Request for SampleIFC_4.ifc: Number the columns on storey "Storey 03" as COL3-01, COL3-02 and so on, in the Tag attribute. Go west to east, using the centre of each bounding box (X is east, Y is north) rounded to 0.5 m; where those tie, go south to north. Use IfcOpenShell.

First a look at what the model holds.

```python
import ifcopenshell
import ifcopenshell.util.element
import ifcopenshell.util.placement

model = ifcopenshell.open("SampleIFC_4.ifc")
print(model.schema)
storey = next(s for s in model.by_type("IfcBuildingStorey") if s.Name == "Storey 03")
columns = [e for e in ifcopenshell.util.element.get_decomposition(storey) if e.is_a("IfcColumn")]
for e in sorted(columns, key=lambda e: e.id()):
    origin = ifcopenshell.util.placement.get_local_placement(e.ObjectPlacement)[:3, 3]
    print(e.id(), e.Tag, e.Name, origin.round(2) + 0.0, sep=" | ")
```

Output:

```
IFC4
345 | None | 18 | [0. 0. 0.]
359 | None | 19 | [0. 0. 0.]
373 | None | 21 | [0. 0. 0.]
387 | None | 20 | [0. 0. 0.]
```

```python
import ifcopenshell
import ifcopenshell.geom
import ifcopenshell.util.element
import ifcopenshell.util.shape

model = ifcopenshell.open("SampleIFC_4.ifc")
settings = ifcopenshell.geom.settings()
settings.set("use-world-coords", True)


def centre(element):
    shape = ifcopenshell.geom.create_shape(settings, element)
    return ifcopenshell.util.shape.get_bbox_centroid(shape.geometry)


storey = next(s for s in model.by_type("IfcBuildingStorey") if s.Name == "Storey 03")
columns = [e for e in ifcopenshell.util.element.get_decomposition(storey) if e.is_a("IfcColumn")]

# Insertion points can sit at a corner or the storey origin, so sort by the geometry (in metres).
centres = {e: centre(e) for e in columns}
columns.sort(key=lambda e: (round(centres[e][0] / 0.5), centres[e][1]))

for i, e in enumerate(columns, start=1):
    number = f"COL3-{i:02d}"
    e.Tag = number
    print(e.id(), number)

model.write("SampleIFC_4_v2.ifc")
```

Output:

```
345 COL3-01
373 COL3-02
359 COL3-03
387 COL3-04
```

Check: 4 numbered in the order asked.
